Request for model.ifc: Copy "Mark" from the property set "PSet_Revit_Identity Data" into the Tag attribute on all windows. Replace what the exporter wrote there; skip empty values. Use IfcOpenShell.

First a look at what the model holds.

```python
import ifcopenshell
import ifcopenshell.util.element

model = ifcopenshell.open("model.ifc")
print(model.schema)
windows = model.by_type("IfcWindow")
print(len(windows), "windows")
for e in windows[:8]:
    source = ifcopenshell.util.element.get_pset(e, "PSet_Revit_Identity Data", "Mark")
    target = e.Tag
    print(e.id(), repr(source), repr(target), sep=" | ")
```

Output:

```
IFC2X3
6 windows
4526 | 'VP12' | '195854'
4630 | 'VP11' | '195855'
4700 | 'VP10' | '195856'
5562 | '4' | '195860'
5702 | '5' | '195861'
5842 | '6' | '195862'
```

```python
import ifcopenshell
import ifcopenshell.util.element

model = ifcopenshell.open("model.ifc")

count = 0
for e in model.by_type("IfcWindow"):
    value = ifcopenshell.util.element.get_pset(e, "PSet_Revit_Identity Data", "Mark")
    current = e.Tag
    if not value or not value.strip() or current == value:
        continue
    e.Tag = value
    count += 1

print(count, "windows updated")

model.write("model_edited.ifc")
```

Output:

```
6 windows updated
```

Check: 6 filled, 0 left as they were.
